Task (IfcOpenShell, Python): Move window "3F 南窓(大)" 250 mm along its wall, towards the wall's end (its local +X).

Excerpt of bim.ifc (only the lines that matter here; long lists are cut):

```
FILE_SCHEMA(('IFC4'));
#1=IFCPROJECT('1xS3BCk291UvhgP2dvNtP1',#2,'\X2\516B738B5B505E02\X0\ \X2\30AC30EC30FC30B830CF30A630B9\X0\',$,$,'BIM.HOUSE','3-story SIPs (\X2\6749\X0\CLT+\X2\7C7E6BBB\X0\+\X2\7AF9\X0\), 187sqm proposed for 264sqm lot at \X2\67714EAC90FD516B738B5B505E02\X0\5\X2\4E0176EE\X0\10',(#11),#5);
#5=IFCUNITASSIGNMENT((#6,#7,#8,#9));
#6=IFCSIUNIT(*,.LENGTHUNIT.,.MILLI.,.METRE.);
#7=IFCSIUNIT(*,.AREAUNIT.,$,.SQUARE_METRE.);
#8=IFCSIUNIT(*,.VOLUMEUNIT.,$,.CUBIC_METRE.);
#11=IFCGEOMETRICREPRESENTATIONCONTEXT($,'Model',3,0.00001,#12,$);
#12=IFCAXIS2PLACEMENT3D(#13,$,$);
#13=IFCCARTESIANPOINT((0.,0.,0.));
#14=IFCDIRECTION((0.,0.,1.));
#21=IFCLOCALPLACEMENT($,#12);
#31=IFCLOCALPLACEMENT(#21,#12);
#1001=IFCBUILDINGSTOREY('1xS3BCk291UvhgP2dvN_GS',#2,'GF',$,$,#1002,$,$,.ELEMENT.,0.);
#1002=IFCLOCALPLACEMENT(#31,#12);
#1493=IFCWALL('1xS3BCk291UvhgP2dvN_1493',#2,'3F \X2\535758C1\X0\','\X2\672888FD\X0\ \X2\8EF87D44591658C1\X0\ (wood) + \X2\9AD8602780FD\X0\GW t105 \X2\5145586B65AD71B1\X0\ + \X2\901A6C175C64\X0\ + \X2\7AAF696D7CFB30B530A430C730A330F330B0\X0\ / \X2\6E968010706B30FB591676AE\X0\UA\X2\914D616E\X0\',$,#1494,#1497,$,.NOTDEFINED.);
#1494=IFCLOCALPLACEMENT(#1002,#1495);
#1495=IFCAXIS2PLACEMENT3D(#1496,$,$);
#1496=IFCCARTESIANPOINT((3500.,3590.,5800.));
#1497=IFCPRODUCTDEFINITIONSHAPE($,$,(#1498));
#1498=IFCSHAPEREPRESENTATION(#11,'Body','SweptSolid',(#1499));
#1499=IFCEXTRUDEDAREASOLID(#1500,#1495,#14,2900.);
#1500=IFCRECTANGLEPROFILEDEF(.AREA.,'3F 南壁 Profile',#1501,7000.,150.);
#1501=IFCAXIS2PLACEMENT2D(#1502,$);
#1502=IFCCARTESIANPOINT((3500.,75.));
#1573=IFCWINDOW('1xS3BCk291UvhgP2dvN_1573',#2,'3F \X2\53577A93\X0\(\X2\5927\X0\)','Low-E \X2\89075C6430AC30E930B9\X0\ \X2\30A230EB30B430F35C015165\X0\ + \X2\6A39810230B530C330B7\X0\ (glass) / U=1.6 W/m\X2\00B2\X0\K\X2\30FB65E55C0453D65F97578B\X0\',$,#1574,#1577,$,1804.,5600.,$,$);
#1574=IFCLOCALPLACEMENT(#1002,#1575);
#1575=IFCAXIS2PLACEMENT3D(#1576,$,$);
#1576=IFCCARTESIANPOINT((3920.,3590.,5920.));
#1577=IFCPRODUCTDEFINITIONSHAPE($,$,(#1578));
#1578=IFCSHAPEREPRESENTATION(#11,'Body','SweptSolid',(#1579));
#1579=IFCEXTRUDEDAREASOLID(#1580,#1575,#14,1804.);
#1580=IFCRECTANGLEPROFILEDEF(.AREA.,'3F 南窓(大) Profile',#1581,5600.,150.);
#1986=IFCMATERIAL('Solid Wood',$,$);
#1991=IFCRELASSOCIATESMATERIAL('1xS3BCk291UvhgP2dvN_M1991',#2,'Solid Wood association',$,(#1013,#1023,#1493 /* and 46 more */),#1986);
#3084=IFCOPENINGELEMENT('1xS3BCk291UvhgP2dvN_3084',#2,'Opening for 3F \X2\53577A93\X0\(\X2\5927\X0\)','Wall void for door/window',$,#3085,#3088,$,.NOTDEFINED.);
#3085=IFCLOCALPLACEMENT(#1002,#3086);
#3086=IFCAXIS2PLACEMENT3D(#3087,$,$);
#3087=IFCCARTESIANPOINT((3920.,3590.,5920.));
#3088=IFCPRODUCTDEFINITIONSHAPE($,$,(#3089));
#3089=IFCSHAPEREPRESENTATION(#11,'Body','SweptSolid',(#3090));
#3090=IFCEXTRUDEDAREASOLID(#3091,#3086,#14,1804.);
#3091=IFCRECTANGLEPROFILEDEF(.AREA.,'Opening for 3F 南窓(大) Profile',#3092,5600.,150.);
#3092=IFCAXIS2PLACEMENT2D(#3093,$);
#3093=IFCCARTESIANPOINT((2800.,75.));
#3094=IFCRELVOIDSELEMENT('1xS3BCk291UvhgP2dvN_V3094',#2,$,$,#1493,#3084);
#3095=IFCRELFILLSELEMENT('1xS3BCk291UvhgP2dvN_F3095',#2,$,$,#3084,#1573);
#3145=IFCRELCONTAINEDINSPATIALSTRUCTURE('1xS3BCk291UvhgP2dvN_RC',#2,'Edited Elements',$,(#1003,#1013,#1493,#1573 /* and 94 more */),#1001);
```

```python
import ifcopenshell
import ifcopenshell.api.geometry
import ifcopenshell.util.placement
import ifcopenshell.util.unit

model = ifcopenshell.open("bim.ifc")
unit_scale = ifcopenshell.util.unit.calculate_unit_scale(model)

window = model.by_guid("1xS3BCk291UvhgP2dvN_1573")
opening = window.FillsVoids[0].RelatingOpeningElement
wall = opening.VoidsElements[0].RelatingBuildingElement

wall_matrix = ifcopenshell.util.placement.get_local_placement(wall.ObjectPlacement)
shift = wall_matrix[:3, 0] * 0.25 / unit_scale
before = ifcopenshell.util.placement.get_local_placement(window.ObjectPlacement)[:3, 3].copy()

# The window is not placed relative to its opening, so move both.
for product in (opening, window):
    matrix = ifcopenshell.util.placement.get_local_placement(product.ObjectPlacement)
    matrix[:3, 3] += shift
    ifcopenshell.api.geometry.edit_object_placement(model, product=product, matrix=matrix, is_si=False)

after = ifcopenshell.util.placement.get_local_placement(window.ObjectPlacement)[:3, 3]
print("window moved by", (after - before).round(3) + 0.0)

model.write("bim-out.ifc")
```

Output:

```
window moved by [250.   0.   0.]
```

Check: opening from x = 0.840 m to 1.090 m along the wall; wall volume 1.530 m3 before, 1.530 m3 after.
